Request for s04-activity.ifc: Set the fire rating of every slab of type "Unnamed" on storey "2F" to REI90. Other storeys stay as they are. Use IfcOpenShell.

First a look at what the model holds.

```python
import ifcopenshell
import ifcopenshell.util.element

model = ifcopenshell.open("s04-activity.ifc")
print(model.schema)
storey = next(s for s in model.by_type("IfcBuildingStorey") if s.Name == "2F")
slabs = [e for e in ifcopenshell.util.element.get_decomposition(storey) if e.is_a("IfcSlab")]
seen = {}
for e in slabs:
    element_type = ifcopenshell.util.element.get_type(e)
    key = (element_type.Name if element_type != e and element_type else None, ifcopenshell.util.element.get_pset(e, "Pset_SlabCommon", "FireRating"))
    seen[key] = seen.get(key, 0) + 1
for (name, value), count in sorted(seen.items(), key=str):
    print(count, "x", name, "|", value)
```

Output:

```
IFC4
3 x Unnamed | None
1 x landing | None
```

```python
import ifcopenshell
import ifcopenshell.api.pset
import ifcopenshell.util.element

model = ifcopenshell.open("s04-activity.ifc")

storey = next(s for s in model.by_type("IfcBuildingStorey") if s.Name == "2F")
slabs = [e for e in ifcopenshell.util.element.get_decomposition(storey) if e.is_a("IfcSlab")]

count = 0
for e in slabs:
    element_type = ifcopenshell.util.element.get_type(e)
    if element_type in (None, e) or element_type.Name != "Unnamed":
        continue
    # add_pset returns the element's existing set when there is one.
    pset = ifcopenshell.api.pset.add_pset(model, product=e, name="Pset_SlabCommon")
    ifcopenshell.api.pset.edit_pset(model, pset=pset, properties={"FireRating": "REI90"})
    count += 1

print(count, "slabs updated")

model.write("s04-activity-out.ifc")
```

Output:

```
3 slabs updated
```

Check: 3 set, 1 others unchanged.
